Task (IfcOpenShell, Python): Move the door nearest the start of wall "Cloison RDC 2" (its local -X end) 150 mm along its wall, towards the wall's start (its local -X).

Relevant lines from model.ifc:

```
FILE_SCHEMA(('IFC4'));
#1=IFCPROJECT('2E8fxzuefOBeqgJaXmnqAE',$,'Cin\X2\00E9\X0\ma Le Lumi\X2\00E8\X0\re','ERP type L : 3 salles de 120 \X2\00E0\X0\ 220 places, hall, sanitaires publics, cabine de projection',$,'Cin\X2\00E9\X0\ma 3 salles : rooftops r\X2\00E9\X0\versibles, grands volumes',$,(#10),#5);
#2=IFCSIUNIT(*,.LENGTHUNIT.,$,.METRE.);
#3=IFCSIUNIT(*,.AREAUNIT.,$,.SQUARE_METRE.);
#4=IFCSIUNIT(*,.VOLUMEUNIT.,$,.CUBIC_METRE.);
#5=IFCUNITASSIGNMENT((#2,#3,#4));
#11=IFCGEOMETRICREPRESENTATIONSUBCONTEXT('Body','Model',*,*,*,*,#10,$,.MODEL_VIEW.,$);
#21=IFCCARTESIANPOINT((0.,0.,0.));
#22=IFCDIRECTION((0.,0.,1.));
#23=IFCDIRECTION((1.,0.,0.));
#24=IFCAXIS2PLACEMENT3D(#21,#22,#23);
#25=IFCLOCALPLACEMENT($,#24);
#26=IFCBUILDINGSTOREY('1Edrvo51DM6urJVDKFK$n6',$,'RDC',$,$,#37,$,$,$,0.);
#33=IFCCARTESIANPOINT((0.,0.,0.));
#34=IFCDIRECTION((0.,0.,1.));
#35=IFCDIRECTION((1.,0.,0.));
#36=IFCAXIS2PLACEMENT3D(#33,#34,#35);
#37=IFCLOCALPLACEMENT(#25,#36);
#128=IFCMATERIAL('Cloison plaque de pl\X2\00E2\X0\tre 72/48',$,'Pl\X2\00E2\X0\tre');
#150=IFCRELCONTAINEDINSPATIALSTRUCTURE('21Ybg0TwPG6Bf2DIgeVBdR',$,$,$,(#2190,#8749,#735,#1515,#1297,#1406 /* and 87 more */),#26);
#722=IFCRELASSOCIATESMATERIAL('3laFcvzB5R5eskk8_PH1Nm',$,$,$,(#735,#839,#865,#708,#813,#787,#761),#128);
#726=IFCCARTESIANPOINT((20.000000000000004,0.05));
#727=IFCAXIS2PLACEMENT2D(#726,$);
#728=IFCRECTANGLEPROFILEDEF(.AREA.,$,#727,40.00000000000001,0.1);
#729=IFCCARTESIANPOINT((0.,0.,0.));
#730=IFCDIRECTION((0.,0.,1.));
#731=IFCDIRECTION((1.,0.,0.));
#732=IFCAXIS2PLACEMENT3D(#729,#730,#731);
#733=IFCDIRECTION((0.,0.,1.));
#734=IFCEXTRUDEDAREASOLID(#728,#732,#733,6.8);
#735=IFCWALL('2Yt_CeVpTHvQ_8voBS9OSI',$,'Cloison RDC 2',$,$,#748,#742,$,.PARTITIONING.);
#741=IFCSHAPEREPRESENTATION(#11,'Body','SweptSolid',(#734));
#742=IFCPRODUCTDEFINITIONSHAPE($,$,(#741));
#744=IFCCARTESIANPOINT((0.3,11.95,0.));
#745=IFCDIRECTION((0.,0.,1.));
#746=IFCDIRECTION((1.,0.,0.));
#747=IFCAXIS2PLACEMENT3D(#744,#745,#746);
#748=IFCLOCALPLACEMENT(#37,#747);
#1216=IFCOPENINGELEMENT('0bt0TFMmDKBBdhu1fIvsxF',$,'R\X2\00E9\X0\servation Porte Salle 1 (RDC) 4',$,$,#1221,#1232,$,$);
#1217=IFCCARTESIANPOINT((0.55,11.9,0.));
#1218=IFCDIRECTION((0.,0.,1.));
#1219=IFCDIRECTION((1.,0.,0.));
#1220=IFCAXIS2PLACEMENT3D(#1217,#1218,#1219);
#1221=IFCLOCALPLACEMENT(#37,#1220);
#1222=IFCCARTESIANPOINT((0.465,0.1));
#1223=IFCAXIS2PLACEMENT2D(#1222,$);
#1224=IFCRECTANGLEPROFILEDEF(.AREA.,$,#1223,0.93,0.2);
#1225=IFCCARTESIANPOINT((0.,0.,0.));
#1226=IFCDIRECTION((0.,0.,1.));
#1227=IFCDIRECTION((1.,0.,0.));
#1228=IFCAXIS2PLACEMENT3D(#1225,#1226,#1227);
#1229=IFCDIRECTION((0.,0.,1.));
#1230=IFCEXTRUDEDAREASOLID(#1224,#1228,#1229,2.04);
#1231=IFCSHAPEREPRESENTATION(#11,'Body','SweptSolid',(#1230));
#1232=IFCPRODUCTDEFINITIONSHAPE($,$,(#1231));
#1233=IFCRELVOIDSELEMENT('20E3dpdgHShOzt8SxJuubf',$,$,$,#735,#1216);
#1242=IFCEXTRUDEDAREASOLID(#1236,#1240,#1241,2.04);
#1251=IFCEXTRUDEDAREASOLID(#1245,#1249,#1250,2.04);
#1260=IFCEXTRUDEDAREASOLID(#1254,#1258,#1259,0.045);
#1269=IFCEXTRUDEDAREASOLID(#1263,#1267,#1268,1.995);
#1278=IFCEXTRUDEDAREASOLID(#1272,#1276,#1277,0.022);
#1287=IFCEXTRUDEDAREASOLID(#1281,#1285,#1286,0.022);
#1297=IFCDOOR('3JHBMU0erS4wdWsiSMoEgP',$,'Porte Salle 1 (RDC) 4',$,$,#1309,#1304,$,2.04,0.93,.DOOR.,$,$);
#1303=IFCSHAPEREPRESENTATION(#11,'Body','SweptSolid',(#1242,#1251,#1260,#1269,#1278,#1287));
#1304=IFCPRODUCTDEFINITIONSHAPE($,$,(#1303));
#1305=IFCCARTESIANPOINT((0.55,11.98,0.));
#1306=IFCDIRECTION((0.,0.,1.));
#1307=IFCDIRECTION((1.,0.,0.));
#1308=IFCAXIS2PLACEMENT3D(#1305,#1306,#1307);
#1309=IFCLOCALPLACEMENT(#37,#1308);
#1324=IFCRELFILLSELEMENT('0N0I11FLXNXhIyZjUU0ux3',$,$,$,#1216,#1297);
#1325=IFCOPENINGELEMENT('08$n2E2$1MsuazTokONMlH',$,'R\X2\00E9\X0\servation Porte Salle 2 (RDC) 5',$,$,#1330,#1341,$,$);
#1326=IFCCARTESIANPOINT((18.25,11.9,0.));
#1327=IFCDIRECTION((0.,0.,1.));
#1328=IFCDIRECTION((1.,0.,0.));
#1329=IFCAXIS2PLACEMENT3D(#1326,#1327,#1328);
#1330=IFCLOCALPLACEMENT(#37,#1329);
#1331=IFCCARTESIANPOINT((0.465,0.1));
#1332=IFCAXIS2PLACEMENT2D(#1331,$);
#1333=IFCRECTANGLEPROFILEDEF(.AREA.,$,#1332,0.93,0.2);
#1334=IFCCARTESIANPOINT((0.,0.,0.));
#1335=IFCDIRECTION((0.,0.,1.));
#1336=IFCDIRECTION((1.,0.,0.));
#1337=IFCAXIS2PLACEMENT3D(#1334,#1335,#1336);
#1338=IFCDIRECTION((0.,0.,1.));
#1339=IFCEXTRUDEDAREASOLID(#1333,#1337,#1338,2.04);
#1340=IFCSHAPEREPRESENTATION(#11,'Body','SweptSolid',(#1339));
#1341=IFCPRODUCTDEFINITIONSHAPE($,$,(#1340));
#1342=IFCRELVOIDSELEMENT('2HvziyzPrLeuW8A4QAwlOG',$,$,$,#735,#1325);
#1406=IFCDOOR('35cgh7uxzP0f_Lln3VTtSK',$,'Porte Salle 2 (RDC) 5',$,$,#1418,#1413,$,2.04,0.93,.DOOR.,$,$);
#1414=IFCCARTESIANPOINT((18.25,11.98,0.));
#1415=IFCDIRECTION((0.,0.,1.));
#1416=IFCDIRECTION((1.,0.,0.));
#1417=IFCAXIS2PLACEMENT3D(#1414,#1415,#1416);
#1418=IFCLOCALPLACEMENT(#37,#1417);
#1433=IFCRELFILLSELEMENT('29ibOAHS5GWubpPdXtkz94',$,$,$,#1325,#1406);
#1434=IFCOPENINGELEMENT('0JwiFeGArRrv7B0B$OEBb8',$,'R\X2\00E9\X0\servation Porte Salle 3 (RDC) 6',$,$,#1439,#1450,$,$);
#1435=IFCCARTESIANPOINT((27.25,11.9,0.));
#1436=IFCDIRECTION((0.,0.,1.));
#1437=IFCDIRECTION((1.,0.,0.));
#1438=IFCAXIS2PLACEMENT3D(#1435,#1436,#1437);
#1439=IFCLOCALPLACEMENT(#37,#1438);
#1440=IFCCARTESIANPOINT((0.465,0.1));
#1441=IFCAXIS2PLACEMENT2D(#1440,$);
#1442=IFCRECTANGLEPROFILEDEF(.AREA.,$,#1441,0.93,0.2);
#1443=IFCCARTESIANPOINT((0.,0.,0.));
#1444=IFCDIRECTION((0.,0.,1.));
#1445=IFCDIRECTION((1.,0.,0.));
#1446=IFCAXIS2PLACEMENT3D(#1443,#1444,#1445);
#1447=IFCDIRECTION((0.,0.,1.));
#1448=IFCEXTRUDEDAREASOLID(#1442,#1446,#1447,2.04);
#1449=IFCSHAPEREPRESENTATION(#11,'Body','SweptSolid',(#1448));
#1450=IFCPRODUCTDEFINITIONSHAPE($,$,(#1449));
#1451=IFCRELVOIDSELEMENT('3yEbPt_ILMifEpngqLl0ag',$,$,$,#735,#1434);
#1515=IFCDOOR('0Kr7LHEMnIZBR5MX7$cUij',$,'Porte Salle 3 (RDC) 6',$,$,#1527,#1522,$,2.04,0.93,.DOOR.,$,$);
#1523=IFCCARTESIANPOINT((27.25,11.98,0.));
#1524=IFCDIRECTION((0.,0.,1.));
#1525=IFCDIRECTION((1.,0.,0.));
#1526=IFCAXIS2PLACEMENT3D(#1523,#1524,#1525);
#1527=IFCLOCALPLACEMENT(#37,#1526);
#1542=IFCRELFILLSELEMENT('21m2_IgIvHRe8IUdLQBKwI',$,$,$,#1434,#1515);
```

```python
import ifcopenshell
import ifcopenshell.api.geometry
import ifcopenshell.util.placement
import ifcopenshell.util.unit

model = ifcopenshell.open("model.ifc")
unit_scale = ifcopenshell.util.unit.calculate_unit_scale(model)

door = model.by_id(1297)
opening = door.FillsVoids[0].RelatingOpeningElement
wall = opening.VoidsElements[0].RelatingBuildingElement

wall_matrix = ifcopenshell.util.placement.get_local_placement(wall.ObjectPlacement)
shift = wall_matrix[:3, 0] * -0.15 / unit_scale
before = ifcopenshell.util.placement.get_local_placement(door.ObjectPlacement)[:3, 3].copy()

# The door is not placed relative to its opening, so move both.
for product in (opening, door):
    matrix = ifcopenshell.util.placement.get_local_placement(product.ObjectPlacement)
    matrix[:3, 3] += shift
    ifcopenshell.api.geometry.edit_object_placement(model, product=product, matrix=matrix, is_si=False)

after = ifcopenshell.util.placement.get_local_placement(door.ObjectPlacement)[:3, 3]
print("door moved by", (after - before).round(3) + 0.0)

model.write("model_rev.ifc")
```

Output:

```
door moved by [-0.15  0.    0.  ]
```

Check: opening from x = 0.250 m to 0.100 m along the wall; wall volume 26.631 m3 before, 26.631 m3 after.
